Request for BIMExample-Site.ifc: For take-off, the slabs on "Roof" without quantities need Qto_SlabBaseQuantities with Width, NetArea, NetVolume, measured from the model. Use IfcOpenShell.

First a look at what the model holds.

```python
import ifcopenshell
import ifcopenshell.util.element
import ifcopenshell.util.unit

model = ifcopenshell.open("BIMExample-Site.ifc")
print(model.schema)
for unit_type in ("LENGTHUNIT", "AREAUNIT", "VOLUMEUNIT"):
    print(unit_type, ifcopenshell.util.unit.calculate_unit_scale(model, unit_type))
storey = next(s for s in model.by_type("IfcBuildingStorey") if s.Name == "Roof")
slabs = [e for e in ifcopenshell.util.element.get_decomposition(storey) if e.is_a("IfcSlab")]
for e in sorted(slabs, key=lambda e: e.id()):
    print(e.id(), e.is_a(), e.Name, list(ifcopenshell.util.element.get_psets(e, qtos_only=True)), sep=" | ")
```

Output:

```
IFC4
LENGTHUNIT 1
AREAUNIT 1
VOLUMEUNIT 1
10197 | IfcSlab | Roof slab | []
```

```python
import ifcopenshell
import ifcopenshell.api.pset
import ifcopenshell.geom
import ifcopenshell.util.element
import ifcopenshell.util.shape
import ifcopenshell.util.unit

model = ifcopenshell.open("BIMExample-Site.ifc")
unit_scale = ifcopenshell.util.unit.calculate_unit_scale(model)
area_scale = ifcopenshell.util.unit.calculate_unit_scale(model, "AREAUNIT")
volume_scale = ifcopenshell.util.unit.calculate_unit_scale(model, "VOLUMEUNIT")
settings = ifcopenshell.geom.settings()

storey = next(s for s in model.by_type("IfcBuildingStorey") if s.Name == "Roof")
slabs = [e for e in ifcopenshell.util.element.get_decomposition(storey) if e.is_a("IfcSlab")]

for e in sorted(slabs, key=lambda e: e.id()):
    if ifcopenshell.util.element.get_psets(e, qtos_only=True, should_inherit=False):
        continue
    # Geometry comes back in metres, in the element's own axes.
    shape = ifcopenshell.geom.create_shape(settings, e)
    values = {
        "Width": ifcopenshell.util.shape.get_z(shape.geometry) / unit_scale,
        "NetArea": ifcopenshell.util.shape.get_footprint_area(shape.geometry) / area_scale,
        "NetVolume": ifcopenshell.util.shape.get_volume(shape.geometry) / volume_scale,
    }
    qto = ifcopenshell.api.pset.add_qto(model, product=e, name="Qto_SlabBaseQuantities")
    ifcopenshell.api.pset.edit_qto(model, qto=qto, properties=values)
    print(e.id(), {k: round(v, 3) for k, v in values.items()})

model.write("BIMExample-Site_edited.ifc")
```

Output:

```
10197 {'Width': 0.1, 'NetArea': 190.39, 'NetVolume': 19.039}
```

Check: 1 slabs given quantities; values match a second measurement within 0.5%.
